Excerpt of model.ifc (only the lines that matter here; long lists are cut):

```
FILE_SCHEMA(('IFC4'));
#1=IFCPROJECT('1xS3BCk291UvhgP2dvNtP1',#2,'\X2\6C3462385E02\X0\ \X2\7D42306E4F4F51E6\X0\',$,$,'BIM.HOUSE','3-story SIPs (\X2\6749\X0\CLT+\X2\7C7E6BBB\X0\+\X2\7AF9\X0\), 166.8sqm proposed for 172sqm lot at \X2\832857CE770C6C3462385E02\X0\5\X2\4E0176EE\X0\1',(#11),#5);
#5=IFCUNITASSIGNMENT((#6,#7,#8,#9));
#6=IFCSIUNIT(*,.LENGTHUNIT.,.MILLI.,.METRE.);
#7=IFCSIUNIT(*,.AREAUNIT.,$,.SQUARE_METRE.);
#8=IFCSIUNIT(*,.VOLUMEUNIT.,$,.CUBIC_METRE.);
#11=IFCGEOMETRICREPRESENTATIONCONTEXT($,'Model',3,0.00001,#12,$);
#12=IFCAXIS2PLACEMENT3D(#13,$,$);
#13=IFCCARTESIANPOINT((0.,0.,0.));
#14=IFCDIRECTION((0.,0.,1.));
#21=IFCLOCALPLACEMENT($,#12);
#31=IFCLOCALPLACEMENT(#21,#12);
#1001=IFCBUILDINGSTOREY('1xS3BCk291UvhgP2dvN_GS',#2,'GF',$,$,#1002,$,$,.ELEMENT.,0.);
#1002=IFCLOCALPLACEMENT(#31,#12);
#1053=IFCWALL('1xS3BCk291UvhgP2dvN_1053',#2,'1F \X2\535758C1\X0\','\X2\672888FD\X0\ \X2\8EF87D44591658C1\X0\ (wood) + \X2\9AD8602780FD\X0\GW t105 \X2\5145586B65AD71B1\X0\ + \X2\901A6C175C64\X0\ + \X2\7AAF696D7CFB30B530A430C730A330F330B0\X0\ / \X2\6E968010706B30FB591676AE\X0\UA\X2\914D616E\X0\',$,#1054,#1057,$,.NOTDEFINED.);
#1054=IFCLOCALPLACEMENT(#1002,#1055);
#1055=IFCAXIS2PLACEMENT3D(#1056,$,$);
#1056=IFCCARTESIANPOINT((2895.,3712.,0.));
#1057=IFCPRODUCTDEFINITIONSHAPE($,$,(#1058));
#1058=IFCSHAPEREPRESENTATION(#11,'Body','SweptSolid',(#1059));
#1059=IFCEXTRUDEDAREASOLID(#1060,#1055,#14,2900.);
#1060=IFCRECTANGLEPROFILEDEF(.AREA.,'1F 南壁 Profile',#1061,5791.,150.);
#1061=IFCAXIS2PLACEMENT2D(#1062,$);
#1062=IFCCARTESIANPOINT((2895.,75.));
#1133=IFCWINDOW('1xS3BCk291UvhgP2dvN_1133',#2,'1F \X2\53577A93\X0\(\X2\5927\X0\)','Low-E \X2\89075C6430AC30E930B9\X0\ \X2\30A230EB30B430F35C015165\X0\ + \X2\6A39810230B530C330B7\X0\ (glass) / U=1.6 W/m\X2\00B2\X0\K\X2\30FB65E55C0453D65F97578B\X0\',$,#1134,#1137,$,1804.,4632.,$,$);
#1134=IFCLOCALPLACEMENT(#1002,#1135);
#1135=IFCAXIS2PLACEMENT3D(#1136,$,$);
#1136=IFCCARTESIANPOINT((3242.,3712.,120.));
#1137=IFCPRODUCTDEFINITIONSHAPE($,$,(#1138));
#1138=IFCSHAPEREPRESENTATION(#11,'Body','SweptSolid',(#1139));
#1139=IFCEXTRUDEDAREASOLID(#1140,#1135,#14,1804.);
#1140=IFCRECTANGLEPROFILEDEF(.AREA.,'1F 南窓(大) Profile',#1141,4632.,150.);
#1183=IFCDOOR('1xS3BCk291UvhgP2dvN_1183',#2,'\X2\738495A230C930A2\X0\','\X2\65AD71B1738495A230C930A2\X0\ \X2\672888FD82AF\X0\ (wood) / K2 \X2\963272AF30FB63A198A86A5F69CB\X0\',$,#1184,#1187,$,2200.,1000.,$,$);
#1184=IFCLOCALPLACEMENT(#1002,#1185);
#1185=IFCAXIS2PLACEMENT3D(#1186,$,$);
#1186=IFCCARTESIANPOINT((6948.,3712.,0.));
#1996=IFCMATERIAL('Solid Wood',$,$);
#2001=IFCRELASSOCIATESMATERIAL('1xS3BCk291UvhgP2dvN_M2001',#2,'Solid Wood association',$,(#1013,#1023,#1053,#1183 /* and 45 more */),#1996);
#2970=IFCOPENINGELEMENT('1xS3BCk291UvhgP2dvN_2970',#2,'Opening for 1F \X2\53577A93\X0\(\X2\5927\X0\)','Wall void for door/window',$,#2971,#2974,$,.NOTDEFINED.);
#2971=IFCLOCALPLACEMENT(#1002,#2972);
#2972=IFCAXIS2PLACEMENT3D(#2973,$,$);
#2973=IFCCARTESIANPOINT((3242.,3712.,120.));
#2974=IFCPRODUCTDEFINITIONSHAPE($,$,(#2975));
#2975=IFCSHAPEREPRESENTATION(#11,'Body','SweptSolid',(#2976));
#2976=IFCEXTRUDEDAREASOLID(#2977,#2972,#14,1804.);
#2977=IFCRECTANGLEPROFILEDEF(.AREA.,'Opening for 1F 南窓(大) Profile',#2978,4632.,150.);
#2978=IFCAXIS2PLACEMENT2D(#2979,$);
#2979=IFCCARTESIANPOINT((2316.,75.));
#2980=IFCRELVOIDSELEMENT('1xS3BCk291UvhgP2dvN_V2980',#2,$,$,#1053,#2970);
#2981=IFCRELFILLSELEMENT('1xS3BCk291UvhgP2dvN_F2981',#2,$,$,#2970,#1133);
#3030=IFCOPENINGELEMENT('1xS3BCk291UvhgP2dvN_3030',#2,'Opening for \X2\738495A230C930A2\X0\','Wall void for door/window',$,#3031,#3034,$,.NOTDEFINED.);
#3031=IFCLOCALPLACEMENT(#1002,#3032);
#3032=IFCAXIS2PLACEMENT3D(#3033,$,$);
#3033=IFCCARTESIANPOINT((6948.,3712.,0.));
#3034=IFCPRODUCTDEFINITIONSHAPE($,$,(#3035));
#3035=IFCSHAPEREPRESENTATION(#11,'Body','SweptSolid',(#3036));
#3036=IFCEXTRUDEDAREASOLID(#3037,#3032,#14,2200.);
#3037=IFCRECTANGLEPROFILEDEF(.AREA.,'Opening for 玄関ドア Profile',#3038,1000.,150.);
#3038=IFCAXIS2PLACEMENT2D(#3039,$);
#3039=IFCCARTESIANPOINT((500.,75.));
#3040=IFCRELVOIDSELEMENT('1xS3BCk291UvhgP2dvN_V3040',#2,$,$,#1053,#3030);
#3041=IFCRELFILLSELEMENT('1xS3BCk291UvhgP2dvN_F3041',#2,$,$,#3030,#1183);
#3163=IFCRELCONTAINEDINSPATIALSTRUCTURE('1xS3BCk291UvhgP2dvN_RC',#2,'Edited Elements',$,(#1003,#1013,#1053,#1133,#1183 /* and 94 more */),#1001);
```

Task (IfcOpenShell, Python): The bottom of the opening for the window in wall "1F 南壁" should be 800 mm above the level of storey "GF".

```python
import numpy as np
import ifcopenshell
import ifcopenshell.api.geometry
import ifcopenshell.geom
import ifcopenshell.util.element
import ifcopenshell.util.placement
import ifcopenshell.util.shape
import ifcopenshell.util.unit

model = ifcopenshell.open("model.ifc")
unit_scale = ifcopenshell.util.unit.calculate_unit_scale(model)

window = model.by_id(1133)
opening = window.FillsVoids[0].RelatingOpeningElement
storey = ifcopenshell.util.element.get_container(window, ifc_class="IfcBuildingStorey")
level = ifcopenshell.util.placement.get_local_placement(storey.ObjectPlacement)[2, 3]

# The opening's origin need not be at the sill, so measure its lowest point.
shape = ifcopenshell.geom.create_shape(ifcopenshell.geom.settings(), opening)
bottom = ifcopenshell.util.shape.get_shape_bottom_elevation(shape, shape.geometry) / unit_scale
dz = level + 0.8 / unit_scale - bottom

shift = np.array([0.0, 0.0, dz])
# The window is not placed relative to its opening, so move both.
for product in (opening, window):
    matrix = ifcopenshell.util.placement.get_local_placement(product.ObjectPlacement)
    matrix[:3, 3] += shift
    ifcopenshell.api.geometry.edit_object_placement(model, product=product, matrix=matrix, is_si=False)

print(f"moved by {dz * unit_scale:+.3f} m")

model.write("model-out.ifc")
```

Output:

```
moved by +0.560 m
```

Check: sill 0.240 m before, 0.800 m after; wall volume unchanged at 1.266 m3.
